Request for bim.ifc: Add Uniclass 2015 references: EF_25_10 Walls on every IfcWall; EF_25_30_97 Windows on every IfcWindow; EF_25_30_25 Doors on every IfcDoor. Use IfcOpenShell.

First a look at what the model holds.

```python
import ifcopenshell

model = ifcopenshell.open("bim.ifc")
print(model.schema)
print("classifications:", [c.Name for c in model.by_type("IfcClassification")])
for ifc_class in ("IfcDoor", "IfcRoof", "IfcStair", "IfcWall", "IfcWindow"):
    print(ifc_class, len(model.by_type(ifc_class)))
```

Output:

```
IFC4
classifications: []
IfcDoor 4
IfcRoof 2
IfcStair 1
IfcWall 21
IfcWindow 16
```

```python
import ifcopenshell
import ifcopenshell.api.classification

model = ifcopenshell.open("bim.ifc")

system = ifcopenshell.api.classification.add_classification(model, classification="Uniclass 2015")

codes = {
    "IfcWall": ("EF_25_10", "Walls"),
    "IfcWindow": ("EF_25_30_97", "Windows"),
    "IfcDoor": ("EF_25_30_25", "Doors"),
}
for ifc_class, (code, name) in codes.items():
    products = model.by_type(ifc_class)
    ifcopenshell.api.classification.add_reference(
        model, products=products, classification=system, identification=code, name=name
    )
    print(code, len(products))

model.write("bim-out.ifc")
```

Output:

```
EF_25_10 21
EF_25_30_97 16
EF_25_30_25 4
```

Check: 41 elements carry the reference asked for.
